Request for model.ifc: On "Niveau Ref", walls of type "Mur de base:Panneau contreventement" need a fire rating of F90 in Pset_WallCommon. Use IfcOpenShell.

First a look at what the model holds.

```python
import ifcopenshell
import ifcopenshell.util.element

model = ifcopenshell.open("model.ifc")
print(model.schema)
storey = next(s for s in model.by_type("IfcBuildingStorey") if s.Name == "Niveau Ref")
walls = [e for e in ifcopenshell.util.element.get_decomposition(storey) if e.is_a("IfcWall")]
seen = {}
for e in walls:
    element_type = ifcopenshell.util.element.get_type(e)
    key = (element_type.Name if element_type != e and element_type else None, ifcopenshell.util.element.get_pset(e, "Pset_WallCommon", "FireRating"))
    seen[key] = seen.get(key, 0) + 1
for (name, value), count in sorted(seen.items(), key=str):
    print(count, "x", name, "|", value)
```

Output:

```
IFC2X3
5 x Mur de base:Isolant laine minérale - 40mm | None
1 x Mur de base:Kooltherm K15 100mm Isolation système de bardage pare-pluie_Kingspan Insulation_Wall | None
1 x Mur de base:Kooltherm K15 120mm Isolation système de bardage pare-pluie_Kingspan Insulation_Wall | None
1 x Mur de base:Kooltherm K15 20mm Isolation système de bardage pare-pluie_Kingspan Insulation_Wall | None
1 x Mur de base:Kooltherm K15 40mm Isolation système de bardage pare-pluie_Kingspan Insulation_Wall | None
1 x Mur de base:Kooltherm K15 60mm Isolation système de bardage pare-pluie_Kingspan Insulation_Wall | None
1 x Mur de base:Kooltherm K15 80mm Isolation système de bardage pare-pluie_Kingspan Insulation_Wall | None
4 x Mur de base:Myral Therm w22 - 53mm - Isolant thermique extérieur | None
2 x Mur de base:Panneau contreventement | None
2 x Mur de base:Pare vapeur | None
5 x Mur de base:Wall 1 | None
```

```python
import ifcopenshell
import ifcopenshell.api.pset
import ifcopenshell.util.element

model = ifcopenshell.open("model.ifc")

storey = next(s for s in model.by_type("IfcBuildingStorey") if s.Name == "Niveau Ref")
walls = [e for e in ifcopenshell.util.element.get_decomposition(storey) if e.is_a("IfcWall")]

count = 0
for e in walls:
    element_type = ifcopenshell.util.element.get_type(e)
    if element_type in (None, e) or element_type.Name != "Mur de base:Panneau contreventement":
        continue
    # add_pset returns the element's existing set when there is one.
    pset = ifcopenshell.api.pset.add_pset(model, product=e, name="Pset_WallCommon")
    ifcopenshell.api.pset.edit_pset(model, pset=pset, properties={"FireRating": "F90"})
    count += 1

print(count, "walls updated")

model.write("model_updated.ifc")
```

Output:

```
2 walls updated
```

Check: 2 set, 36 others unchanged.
